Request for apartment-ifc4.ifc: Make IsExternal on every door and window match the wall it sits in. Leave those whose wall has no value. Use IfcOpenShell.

First a look at what the model holds.

```python
import ifcopenshell
import ifcopenshell.util.element

model = ifcopenshell.open("apartment-ifc4.ifc")
print(model.schema)
seen = {}
for e in model.by_type("IfcDoor") + model.by_type("IfcWindow"):
    if not e.FillsVoids:
        continue
    host = e.FillsVoids[0].RelatingOpeningElement.VoidsElements[0].RelatingBuildingElement
    own = ifcopenshell.util.element.get_pset(e, f"Pset_{e.is_a()[3:].removesuffix('StandardCase')}Common", "IsExternal")
    wall = ifcopenshell.util.element.get_pset(host, "Pset_WallCommon", "IsExternal")
    seen[e.is_a(), own, wall] = seen.get((e.is_a(), own, wall), 0) + 1
for (cls, own, wall), count in sorted(seen.items(), key=str):
    print(count, cls, "IsExternal:", own, "| host wall:", wall)
```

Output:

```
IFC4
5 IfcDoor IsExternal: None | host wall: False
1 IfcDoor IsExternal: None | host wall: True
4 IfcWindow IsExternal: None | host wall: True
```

```python
import ifcopenshell
import ifcopenshell.api.pset
import ifcopenshell.util.element

model = ifcopenshell.open("apartment-ifc4.ifc")

count = 0
for ifc_class, pset_name in (("IfcDoor", "Pset_DoorCommon"), ("IfcWindow", "Pset_WindowCommon")):
    for e in model.by_type(ifc_class):
        if not e.FillsVoids:
            continue
        host = e.FillsVoids[0].RelatingOpeningElement.VoidsElements[0].RelatingBuildingElement
        external = ifcopenshell.util.element.get_pset(host, "Pset_WallCommon", "IsExternal")
        if external is None or ifcopenshell.util.element.get_pset(e, pset_name, "IsExternal") == external:
            continue
        pset = ifcopenshell.api.pset.add_pset(model, product=e, name=pset_name)
        ifcopenshell.api.pset.edit_pset(model, pset=pset, properties={"IsExternal": external})
        count += 1

print(count, "updated")

model.write("apartment-ifc4_edited.ifc")
```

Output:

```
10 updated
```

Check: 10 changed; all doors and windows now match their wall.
